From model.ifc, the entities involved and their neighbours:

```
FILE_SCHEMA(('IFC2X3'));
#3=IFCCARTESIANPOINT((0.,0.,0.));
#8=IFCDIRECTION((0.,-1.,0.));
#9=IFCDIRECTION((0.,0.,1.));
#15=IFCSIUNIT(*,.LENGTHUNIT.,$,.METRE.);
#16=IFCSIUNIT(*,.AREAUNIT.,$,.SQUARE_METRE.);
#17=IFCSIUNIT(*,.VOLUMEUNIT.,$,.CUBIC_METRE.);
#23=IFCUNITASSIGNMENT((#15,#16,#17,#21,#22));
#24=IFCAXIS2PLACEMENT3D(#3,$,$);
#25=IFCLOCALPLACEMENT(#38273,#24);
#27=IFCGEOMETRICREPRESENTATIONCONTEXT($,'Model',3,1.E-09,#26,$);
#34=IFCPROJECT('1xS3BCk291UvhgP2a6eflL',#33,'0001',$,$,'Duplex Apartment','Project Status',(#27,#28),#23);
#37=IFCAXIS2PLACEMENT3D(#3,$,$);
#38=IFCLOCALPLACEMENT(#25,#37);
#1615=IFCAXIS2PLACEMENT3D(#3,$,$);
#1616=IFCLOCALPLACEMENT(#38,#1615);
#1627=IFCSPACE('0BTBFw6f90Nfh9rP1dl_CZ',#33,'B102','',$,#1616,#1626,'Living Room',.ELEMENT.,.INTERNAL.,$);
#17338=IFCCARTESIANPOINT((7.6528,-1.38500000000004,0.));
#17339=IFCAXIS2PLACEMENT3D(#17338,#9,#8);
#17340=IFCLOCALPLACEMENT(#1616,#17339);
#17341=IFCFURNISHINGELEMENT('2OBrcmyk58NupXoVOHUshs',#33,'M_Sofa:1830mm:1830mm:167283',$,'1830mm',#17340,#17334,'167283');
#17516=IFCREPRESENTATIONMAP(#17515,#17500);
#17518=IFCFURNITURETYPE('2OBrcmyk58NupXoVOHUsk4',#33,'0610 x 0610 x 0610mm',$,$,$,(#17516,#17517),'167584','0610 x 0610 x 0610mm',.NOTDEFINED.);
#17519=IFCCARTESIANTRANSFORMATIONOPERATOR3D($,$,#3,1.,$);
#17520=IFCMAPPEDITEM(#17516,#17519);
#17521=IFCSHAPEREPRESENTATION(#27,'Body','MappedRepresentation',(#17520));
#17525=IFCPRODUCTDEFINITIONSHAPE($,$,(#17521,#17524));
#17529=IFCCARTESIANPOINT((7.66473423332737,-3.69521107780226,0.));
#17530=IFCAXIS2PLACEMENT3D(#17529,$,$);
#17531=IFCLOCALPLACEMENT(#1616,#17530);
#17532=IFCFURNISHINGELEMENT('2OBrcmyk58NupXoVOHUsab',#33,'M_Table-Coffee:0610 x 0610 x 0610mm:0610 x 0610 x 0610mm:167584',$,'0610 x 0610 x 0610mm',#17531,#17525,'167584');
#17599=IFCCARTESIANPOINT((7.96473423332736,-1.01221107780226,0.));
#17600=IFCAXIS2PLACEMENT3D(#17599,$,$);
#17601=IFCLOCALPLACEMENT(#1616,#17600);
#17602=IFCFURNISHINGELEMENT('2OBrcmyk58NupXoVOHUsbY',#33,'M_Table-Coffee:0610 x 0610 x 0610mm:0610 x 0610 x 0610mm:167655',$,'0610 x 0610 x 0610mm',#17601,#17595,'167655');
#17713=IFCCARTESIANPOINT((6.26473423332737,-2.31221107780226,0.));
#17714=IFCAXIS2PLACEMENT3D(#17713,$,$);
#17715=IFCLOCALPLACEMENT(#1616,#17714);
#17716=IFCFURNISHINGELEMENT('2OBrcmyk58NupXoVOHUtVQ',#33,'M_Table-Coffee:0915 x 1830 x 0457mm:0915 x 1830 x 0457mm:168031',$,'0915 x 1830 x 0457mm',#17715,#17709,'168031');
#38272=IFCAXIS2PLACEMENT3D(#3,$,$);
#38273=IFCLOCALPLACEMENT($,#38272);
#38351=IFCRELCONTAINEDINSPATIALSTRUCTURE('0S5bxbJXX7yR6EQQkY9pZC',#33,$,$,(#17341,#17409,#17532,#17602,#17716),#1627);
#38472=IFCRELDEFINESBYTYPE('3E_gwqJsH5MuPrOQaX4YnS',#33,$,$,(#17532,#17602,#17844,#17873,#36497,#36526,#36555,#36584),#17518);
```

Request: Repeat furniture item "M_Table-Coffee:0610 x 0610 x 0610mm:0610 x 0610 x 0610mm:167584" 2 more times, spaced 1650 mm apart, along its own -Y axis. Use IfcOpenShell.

```python
import ifcopenshell
import ifcopenshell.api.geometry
import ifcopenshell.api.root
import ifcopenshell.util.element
import ifcopenshell.util.placement

model = ifcopenshell.open("model.ifc")


def reuse_history(source, copy):
    """copy_class also copies each property set's owner history, people and application; keep the originals."""
    for rel in copy.IsDefinedBy:
        if rel.is_a("IfcRelDefinesByProperties") and (history := rel.RelatingPropertyDefinition.OwnerHistory):
            rel.RelatingPropertyDefinition.OwnerHistory = source.OwnerHistory
            ifcopenshell.util.element.remove_deep2(model, history)


source = model.by_guid("2OBrcmyk58NupXoVOHUsab")
base = ifcopenshell.util.placement.get_local_placement(source.ObjectPlacement)
step = -base[:3, 1] * 1.65

for i in range(1, 3):
    copy = ifcopenshell.api.root.copy_class(model, product=source)
    copy.Representation = ifcopenshell.util.element.copy_deep(
        model, source.Representation, exclude=["IfcGeometricRepresentationContext", "IfcRepresentationMap"]
    )
    copy.Name = "M_Table-Coffee:0610 x 0610 x 0610mm:0610 x 0610 x 0610mm"
    copy.Tag = None
    reuse_history(source, copy)
    matrix = base.copy()
    matrix[:3, 3] += i * step
    print("added at", matrix[:3, 3].round(3) + 0.0)
    ifcopenshell.api.geometry.edit_object_placement(model, product=copy, matrix=matrix, is_si=False)

model.write("model_edited.ifc")
```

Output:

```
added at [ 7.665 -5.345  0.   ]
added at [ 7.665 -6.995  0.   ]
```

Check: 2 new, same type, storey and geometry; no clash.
